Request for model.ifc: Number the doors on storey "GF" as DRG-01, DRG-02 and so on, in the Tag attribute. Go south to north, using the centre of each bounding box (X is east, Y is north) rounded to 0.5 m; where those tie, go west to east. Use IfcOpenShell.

First a look at what the model holds.

```python
import ifcopenshell
import ifcopenshell.util.element
import ifcopenshell.util.placement

model = ifcopenshell.open("model.ifc")
print(model.schema)
storey = next(s for s in model.by_type("IfcBuildingStorey") if s.Name == "GF")
doors = [e for e in ifcopenshell.util.element.get_decomposition(storey) if e.is_a("IfcDoor")]
for e in sorted(doors, key=lambda e: e.id()):
    origin = ifcopenshell.util.placement.get_local_placement(e.ObjectPlacement)[:3, 3]
    print(e.id(), e.Tag, e.Name, origin.round(2) + 0.0, sep=" | ")
```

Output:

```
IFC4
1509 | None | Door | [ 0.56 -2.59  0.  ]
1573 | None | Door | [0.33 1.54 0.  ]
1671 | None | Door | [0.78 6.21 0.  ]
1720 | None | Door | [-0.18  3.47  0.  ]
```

```python
import ifcopenshell
import ifcopenshell.geom
import ifcopenshell.util.element
import ifcopenshell.util.shape

model = ifcopenshell.open("model.ifc")
settings = ifcopenshell.geom.settings()
settings.set("use-world-coords", True)


def centre(element):
    shape = ifcopenshell.geom.create_shape(settings, element)
    return ifcopenshell.util.shape.get_bbox_centroid(shape.geometry)


storey = next(s for s in model.by_type("IfcBuildingStorey") if s.Name == "GF")
doors = [e for e in ifcopenshell.util.element.get_decomposition(storey) if e.is_a("IfcDoor")]

# Insertion points can sit at a corner or the storey origin, so sort by the geometry (in metres).
centres = {e: centre(e) for e in doors}
doors.sort(key=lambda e: (round(centres[e][1] / 0.5), centres[e][0]))

for i, e in enumerate(doors, start=1):
    number = f"DRG-{i:02d}"
    e.Tag = number
    print(e.id(), number)

model.write("model_rev.ifc")
```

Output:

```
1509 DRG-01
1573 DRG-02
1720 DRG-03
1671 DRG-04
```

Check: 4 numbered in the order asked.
